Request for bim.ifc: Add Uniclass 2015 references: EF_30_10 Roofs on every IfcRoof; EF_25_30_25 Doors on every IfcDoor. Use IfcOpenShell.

First a look at what the model holds.

```python
import ifcopenshell

model = ifcopenshell.open("bim.ifc")
print(model.schema)
print("classifications:", [c.Name for c in model.by_type("IfcClassification")])
for ifc_class in ("IfcDoor", "IfcRoof", "IfcStair", "IfcWall", "IfcWindow"):
    print(ifc_class, len(model.by_type(ifc_class)))
```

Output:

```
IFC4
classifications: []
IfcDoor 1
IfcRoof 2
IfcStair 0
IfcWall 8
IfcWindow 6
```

```python
import ifcopenshell
import ifcopenshell.api.classification

model = ifcopenshell.open("bim.ifc")

system = ifcopenshell.api.classification.add_classification(model, classification="Uniclass 2015")

codes = {
    "IfcRoof": ("EF_30_10", "Roofs"),
    "IfcDoor": ("EF_25_30_25", "Doors"),
}
for ifc_class, (code, name) in codes.items():
    products = model.by_type(ifc_class)
    ifcopenshell.api.classification.add_reference(
        model, products=products, classification=system, identification=code, name=name
    )
    print(code, len(products))

model.write("bim_edited.ifc")
```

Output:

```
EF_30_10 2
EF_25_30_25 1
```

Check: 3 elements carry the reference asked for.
